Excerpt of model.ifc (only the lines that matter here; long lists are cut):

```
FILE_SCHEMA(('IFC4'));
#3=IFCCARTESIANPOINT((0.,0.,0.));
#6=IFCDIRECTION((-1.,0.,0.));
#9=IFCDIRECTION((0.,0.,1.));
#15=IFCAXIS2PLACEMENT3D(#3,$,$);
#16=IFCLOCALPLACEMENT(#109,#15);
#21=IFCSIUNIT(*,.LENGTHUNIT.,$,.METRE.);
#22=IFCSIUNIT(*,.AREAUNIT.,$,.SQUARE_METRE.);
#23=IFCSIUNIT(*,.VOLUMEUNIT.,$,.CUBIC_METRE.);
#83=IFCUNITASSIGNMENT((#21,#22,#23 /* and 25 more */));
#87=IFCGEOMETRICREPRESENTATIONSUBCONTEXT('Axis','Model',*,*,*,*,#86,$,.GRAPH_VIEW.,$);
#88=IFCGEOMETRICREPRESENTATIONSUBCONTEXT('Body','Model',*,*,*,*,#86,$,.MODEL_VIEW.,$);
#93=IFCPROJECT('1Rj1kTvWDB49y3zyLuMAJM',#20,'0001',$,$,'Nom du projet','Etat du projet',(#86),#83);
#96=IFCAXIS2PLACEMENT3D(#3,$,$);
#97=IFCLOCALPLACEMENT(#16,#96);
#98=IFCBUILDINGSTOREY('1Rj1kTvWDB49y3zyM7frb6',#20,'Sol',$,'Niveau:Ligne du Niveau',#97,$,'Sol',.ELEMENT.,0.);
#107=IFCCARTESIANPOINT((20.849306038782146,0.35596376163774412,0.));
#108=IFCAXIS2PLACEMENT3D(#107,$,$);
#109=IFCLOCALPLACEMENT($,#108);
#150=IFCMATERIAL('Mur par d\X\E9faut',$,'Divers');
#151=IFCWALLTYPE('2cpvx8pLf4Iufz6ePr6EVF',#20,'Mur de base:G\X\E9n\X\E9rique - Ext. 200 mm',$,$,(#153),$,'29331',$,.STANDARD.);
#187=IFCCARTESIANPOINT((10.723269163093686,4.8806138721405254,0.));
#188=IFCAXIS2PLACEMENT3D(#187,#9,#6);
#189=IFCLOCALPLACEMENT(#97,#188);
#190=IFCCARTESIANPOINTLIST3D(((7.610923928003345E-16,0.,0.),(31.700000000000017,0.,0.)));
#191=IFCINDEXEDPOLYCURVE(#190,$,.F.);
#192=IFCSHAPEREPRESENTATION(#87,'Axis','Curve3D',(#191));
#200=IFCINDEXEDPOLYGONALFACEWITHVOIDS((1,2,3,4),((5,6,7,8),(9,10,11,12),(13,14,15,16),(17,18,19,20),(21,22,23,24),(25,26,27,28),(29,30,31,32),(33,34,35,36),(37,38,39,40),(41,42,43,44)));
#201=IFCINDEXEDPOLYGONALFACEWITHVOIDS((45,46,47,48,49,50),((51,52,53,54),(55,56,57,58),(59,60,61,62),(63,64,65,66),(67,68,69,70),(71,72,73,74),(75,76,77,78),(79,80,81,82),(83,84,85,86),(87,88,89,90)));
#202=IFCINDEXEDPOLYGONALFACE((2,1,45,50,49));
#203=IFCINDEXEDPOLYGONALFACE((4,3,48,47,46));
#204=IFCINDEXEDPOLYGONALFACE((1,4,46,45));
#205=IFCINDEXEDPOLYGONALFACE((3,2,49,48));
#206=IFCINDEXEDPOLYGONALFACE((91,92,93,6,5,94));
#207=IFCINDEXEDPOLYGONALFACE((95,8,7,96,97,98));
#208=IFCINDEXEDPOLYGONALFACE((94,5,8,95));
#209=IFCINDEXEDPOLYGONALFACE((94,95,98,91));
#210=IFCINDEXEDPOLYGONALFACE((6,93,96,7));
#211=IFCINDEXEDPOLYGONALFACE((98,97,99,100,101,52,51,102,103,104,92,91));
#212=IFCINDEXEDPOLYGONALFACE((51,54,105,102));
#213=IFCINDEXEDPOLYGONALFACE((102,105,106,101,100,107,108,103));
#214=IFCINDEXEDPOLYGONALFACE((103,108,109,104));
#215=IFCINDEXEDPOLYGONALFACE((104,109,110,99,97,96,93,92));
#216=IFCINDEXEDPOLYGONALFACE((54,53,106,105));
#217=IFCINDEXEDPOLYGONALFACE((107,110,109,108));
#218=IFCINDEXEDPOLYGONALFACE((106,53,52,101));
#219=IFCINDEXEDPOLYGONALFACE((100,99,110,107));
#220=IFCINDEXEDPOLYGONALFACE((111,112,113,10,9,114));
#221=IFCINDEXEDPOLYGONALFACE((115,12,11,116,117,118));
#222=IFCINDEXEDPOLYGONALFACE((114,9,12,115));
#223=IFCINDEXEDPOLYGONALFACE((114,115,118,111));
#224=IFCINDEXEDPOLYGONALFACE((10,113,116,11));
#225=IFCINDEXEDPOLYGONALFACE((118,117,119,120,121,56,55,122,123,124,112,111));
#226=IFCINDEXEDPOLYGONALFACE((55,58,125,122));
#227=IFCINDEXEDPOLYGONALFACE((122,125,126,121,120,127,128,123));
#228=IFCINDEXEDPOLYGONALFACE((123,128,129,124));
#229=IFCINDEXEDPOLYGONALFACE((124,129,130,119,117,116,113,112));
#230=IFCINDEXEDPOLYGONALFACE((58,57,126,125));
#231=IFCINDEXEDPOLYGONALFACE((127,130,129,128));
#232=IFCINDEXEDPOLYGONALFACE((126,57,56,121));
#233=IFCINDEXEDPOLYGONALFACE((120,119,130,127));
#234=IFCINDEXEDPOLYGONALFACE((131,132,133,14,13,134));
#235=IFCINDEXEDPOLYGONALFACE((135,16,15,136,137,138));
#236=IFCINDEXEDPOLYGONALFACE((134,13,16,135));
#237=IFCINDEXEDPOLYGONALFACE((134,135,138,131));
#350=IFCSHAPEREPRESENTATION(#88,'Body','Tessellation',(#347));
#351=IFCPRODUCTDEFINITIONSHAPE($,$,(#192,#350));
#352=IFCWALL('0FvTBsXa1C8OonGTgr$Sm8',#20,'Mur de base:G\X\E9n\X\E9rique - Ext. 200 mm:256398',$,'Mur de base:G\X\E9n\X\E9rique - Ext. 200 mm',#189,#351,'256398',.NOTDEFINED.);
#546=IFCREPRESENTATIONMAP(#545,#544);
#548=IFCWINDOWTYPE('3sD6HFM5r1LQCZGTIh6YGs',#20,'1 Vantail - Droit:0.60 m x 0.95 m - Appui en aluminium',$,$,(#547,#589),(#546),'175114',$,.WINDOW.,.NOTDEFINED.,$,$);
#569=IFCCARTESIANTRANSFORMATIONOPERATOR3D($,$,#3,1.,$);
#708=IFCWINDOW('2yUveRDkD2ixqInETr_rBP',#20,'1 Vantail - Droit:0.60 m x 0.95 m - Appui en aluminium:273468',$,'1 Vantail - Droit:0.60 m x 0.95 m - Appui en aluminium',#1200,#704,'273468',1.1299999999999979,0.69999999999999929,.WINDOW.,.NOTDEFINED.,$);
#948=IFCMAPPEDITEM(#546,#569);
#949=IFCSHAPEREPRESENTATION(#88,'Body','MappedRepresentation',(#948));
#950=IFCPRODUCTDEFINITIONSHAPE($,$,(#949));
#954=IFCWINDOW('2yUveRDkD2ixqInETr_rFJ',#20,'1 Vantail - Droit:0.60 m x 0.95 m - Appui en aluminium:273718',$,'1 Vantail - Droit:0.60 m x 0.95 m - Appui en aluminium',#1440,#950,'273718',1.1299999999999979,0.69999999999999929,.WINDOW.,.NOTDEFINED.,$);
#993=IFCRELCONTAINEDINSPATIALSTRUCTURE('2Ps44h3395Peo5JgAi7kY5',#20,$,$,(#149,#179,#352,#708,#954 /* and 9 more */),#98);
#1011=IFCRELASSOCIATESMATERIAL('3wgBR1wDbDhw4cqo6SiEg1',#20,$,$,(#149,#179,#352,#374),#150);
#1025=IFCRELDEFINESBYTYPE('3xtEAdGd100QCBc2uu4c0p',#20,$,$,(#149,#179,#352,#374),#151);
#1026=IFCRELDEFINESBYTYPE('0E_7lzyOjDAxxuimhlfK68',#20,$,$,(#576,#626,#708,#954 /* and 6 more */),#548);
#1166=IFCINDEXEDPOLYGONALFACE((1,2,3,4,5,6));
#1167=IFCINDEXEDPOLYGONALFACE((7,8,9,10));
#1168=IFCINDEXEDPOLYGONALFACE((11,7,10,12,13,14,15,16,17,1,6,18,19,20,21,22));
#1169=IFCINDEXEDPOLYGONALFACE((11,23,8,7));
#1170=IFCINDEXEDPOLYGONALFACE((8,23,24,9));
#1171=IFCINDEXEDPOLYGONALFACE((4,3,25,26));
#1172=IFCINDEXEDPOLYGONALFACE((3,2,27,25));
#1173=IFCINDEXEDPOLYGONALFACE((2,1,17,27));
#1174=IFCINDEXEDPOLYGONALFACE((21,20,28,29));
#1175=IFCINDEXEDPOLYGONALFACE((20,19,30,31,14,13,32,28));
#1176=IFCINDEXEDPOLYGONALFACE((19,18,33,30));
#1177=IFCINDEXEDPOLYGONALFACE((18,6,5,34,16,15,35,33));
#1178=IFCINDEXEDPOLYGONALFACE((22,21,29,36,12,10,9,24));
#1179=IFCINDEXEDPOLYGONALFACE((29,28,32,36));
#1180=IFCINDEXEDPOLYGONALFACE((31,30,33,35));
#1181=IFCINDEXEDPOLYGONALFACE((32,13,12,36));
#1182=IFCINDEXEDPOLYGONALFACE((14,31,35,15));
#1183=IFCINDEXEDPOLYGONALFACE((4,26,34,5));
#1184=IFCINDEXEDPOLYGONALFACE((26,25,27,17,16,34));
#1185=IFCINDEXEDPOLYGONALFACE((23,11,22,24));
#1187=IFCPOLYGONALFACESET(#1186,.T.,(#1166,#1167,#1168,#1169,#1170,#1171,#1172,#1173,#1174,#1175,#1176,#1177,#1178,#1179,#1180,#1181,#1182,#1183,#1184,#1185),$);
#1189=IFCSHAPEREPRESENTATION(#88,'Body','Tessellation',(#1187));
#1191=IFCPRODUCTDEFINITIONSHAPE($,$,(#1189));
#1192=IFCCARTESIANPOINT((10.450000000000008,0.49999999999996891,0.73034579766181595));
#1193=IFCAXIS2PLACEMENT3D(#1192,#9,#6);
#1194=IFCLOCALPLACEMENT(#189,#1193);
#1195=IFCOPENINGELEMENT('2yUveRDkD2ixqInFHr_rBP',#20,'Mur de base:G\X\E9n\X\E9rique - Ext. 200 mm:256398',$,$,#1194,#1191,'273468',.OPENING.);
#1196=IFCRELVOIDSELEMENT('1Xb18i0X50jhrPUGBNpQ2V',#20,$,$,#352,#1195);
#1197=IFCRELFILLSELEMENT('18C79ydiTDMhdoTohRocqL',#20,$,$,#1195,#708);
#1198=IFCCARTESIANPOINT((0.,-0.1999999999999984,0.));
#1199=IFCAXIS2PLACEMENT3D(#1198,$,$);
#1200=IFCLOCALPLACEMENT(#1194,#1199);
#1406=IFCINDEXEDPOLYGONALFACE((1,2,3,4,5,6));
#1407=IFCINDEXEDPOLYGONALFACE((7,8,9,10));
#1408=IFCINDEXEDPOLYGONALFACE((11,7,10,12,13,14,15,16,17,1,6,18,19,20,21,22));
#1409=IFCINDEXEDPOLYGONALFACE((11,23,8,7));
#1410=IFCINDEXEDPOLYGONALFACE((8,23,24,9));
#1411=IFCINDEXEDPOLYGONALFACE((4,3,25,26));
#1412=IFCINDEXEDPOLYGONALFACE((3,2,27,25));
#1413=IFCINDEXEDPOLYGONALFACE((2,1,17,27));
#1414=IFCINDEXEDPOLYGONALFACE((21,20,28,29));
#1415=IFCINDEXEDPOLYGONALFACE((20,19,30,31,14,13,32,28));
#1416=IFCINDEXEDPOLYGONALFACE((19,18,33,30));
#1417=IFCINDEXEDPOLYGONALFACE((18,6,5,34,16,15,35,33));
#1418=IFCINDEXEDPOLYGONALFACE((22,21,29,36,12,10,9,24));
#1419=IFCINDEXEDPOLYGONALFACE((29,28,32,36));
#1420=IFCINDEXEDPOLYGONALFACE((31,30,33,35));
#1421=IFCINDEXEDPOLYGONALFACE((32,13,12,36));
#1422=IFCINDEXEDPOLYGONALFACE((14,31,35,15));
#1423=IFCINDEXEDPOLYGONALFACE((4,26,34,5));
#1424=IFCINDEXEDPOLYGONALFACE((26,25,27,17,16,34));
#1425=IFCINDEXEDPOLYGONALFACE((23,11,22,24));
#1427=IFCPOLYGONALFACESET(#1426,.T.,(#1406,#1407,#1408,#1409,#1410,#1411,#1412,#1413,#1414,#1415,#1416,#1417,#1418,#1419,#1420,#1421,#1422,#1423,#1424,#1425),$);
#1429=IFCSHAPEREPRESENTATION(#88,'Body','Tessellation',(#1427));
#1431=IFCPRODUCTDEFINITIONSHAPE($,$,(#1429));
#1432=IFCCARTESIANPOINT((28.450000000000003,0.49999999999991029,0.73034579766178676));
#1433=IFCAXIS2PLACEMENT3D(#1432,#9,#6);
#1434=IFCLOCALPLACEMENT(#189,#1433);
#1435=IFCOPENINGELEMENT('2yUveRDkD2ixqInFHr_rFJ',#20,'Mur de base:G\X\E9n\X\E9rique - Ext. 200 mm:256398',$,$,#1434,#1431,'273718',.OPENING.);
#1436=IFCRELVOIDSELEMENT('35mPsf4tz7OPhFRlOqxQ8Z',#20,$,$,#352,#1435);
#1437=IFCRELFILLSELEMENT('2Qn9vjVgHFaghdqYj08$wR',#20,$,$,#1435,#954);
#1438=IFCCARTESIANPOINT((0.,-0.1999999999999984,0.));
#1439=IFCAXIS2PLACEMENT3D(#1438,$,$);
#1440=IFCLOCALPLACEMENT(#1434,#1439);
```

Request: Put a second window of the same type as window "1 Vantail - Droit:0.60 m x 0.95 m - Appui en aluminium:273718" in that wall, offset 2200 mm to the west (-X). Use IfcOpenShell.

```python
import ifcopenshell
import ifcopenshell.api.feature
import ifcopenshell.api.geometry
import ifcopenshell.api.root
import ifcopenshell.geom
import ifcopenshell.util.element
import ifcopenshell.util.placement
import ifcopenshell.util.shape
import ifcopenshell.util.unit

model = ifcopenshell.open("model.ifc")
unit_scale = ifcopenshell.util.unit.calculate_unit_scale(model)
settings = ifcopenshell.geom.settings()


def volume(element):
    """Net volume in cubic metres, openings subtracted."""
    shape = ifcopenshell.geom.create_shape(settings, element)
    return ifcopenshell.util.shape.get_volume(shape.geometry)


def reuse_history(source, copy):
    """copy_class also copies each property set's owner history, people and application; keep the originals."""
    for rel in copy.IsDefinedBy:
        if rel.is_a("IfcRelDefinesByProperties") and (history := rel.RelatingPropertyDefinition.OwnerHistory):
            rel.RelatingPropertyDefinition.OwnerHistory = source.OwnerHistory
            ifcopenshell.util.element.remove_deep2(model, history)


window = model.by_guid("2yUveRDkD2ixqInETr_rFJ")
opening = window.FillsVoids[0].RelatingOpeningElement
wall = opening.VoidsElements[0].RelatingBuildingElement
before = volume(wall)
shift = ifcopenshell.util.placement.get_local_placement(wall.ObjectPlacement)[:3, 0] * 2.2 / unit_scale

# copy_class copies the void relationship, type, container and properties, but no geometry.
new_opening = ifcopenshell.api.root.copy_class(model, product=opening)
new_opening.Representation = ifcopenshell.util.element.copy_deep(
    model, opening.Representation, exclude=["IfcGeometricRepresentationContext", "IfcRepresentationMap"]
)
new_opening.Name = "Mur de base:Générique - Ext. 200 mm"
new_opening.Tag = None
new_window = ifcopenshell.api.root.copy_class(model, product=window)
new_window.Representation = ifcopenshell.util.element.copy_deep(
    model, window.Representation, exclude=["IfcGeometricRepresentationContext", "IfcRepresentationMap"]
)
new_window.Name = "1 Vantail - Droit:0.60 m x 0.95 m - Appui en aluminium"
new_window.Tag = None
reuse_history(window, new_window)
ifcopenshell.api.feature.add_filling(model, opening=new_opening, element=new_window)

for old, new in ((opening, new_opening), (window, new_window)):
    matrix = ifcopenshell.util.placement.get_local_placement(old.ObjectPlacement)
    matrix[:3, 3] += shift
    ifcopenshell.api.geometry.edit_object_placement(model, product=new, matrix=matrix, is_si=False)

after = volume(wall)

print(f"wall volume {before:.3f} -> {after:.3f} m3")

model.write("model_edited.ifc")
```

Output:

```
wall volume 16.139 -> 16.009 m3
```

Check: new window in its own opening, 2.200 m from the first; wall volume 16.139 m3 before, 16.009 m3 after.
